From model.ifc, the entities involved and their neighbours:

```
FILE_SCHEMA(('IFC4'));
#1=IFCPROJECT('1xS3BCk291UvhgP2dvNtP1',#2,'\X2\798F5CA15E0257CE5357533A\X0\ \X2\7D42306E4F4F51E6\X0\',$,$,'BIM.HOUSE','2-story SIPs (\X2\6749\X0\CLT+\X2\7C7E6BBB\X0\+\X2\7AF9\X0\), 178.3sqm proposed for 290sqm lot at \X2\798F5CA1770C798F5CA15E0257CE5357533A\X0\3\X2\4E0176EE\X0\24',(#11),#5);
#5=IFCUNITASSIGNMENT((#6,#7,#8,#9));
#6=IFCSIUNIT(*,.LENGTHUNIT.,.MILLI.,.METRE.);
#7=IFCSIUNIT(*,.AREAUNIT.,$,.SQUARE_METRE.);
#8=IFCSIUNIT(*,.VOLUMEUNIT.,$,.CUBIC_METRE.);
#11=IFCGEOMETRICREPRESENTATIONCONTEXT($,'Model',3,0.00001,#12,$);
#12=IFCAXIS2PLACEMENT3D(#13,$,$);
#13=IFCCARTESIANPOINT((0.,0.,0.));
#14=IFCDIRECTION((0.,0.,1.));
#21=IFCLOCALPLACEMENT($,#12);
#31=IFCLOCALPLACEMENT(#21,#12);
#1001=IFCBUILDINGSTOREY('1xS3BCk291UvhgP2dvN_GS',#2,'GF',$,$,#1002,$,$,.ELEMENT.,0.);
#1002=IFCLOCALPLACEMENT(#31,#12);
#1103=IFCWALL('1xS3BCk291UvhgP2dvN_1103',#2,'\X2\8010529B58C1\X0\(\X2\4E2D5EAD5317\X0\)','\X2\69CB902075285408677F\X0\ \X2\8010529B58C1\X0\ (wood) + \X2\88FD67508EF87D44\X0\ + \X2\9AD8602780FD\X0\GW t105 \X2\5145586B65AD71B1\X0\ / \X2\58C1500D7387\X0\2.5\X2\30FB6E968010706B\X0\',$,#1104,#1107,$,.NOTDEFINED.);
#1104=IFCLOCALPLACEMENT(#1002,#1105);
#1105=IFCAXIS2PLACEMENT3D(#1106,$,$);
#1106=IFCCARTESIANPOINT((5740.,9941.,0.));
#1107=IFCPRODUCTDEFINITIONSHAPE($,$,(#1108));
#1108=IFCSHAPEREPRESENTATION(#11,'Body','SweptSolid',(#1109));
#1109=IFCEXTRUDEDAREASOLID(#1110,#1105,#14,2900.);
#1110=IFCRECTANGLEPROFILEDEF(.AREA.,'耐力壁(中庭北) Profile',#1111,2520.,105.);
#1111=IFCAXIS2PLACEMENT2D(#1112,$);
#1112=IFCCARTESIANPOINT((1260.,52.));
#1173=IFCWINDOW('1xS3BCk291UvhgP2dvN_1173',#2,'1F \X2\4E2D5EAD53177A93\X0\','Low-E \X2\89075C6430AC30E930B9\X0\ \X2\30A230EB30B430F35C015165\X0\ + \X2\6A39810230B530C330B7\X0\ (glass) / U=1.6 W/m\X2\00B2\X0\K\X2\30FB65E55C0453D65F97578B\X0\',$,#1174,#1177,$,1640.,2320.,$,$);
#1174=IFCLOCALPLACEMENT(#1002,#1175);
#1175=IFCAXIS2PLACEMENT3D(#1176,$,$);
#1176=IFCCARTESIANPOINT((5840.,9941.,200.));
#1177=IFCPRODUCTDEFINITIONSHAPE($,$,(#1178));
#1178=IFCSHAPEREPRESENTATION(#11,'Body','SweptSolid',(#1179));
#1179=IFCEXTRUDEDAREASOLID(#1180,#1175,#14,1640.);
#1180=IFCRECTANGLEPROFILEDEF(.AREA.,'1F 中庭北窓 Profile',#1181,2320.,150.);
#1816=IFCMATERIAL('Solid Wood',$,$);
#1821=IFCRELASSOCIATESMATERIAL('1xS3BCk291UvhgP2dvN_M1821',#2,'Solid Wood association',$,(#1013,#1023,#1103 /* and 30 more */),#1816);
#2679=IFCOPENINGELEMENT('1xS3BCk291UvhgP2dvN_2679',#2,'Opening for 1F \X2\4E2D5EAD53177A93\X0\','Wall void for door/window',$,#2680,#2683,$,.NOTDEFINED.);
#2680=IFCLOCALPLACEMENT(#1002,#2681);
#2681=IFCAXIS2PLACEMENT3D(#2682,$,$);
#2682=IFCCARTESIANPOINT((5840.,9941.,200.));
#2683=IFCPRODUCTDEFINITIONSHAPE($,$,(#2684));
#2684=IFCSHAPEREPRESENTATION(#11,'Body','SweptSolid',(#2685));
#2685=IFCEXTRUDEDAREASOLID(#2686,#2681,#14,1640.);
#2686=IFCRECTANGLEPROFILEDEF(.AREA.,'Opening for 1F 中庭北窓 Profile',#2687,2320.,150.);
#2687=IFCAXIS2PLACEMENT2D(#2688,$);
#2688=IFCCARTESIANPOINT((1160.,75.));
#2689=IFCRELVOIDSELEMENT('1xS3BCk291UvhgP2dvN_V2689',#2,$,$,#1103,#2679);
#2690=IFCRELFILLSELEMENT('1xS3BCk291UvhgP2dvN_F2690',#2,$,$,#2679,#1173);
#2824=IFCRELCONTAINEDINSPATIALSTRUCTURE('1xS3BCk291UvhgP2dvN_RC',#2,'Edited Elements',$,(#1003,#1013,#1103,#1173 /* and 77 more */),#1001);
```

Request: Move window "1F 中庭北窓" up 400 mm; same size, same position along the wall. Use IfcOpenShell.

```python
import numpy as np
import ifcopenshell
import ifcopenshell.api.geometry
import ifcopenshell.util.placement
import ifcopenshell.util.unit

model = ifcopenshell.open("model.ifc")
unit_scale = ifcopenshell.util.unit.calculate_unit_scale(model)

window = model.by_id(1173)
opening = window.FillsVoids[0].RelatingOpeningElement
dz = 0.4 / unit_scale

shift = np.array([0.0, 0.0, dz])
# The window is not placed relative to its opening, so move both.
for product in (opening, window):
    matrix = ifcopenshell.util.placement.get_local_placement(product.ObjectPlacement)
    matrix[:3, 3] += shift
    ifcopenshell.api.geometry.edit_object_placement(model, product=product, matrix=matrix, is_si=False)

print(f"moved by {dz * unit_scale:+.3f} m")

model.write("model_updated.ifc")
```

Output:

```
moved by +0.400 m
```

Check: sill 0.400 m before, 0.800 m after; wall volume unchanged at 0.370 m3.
